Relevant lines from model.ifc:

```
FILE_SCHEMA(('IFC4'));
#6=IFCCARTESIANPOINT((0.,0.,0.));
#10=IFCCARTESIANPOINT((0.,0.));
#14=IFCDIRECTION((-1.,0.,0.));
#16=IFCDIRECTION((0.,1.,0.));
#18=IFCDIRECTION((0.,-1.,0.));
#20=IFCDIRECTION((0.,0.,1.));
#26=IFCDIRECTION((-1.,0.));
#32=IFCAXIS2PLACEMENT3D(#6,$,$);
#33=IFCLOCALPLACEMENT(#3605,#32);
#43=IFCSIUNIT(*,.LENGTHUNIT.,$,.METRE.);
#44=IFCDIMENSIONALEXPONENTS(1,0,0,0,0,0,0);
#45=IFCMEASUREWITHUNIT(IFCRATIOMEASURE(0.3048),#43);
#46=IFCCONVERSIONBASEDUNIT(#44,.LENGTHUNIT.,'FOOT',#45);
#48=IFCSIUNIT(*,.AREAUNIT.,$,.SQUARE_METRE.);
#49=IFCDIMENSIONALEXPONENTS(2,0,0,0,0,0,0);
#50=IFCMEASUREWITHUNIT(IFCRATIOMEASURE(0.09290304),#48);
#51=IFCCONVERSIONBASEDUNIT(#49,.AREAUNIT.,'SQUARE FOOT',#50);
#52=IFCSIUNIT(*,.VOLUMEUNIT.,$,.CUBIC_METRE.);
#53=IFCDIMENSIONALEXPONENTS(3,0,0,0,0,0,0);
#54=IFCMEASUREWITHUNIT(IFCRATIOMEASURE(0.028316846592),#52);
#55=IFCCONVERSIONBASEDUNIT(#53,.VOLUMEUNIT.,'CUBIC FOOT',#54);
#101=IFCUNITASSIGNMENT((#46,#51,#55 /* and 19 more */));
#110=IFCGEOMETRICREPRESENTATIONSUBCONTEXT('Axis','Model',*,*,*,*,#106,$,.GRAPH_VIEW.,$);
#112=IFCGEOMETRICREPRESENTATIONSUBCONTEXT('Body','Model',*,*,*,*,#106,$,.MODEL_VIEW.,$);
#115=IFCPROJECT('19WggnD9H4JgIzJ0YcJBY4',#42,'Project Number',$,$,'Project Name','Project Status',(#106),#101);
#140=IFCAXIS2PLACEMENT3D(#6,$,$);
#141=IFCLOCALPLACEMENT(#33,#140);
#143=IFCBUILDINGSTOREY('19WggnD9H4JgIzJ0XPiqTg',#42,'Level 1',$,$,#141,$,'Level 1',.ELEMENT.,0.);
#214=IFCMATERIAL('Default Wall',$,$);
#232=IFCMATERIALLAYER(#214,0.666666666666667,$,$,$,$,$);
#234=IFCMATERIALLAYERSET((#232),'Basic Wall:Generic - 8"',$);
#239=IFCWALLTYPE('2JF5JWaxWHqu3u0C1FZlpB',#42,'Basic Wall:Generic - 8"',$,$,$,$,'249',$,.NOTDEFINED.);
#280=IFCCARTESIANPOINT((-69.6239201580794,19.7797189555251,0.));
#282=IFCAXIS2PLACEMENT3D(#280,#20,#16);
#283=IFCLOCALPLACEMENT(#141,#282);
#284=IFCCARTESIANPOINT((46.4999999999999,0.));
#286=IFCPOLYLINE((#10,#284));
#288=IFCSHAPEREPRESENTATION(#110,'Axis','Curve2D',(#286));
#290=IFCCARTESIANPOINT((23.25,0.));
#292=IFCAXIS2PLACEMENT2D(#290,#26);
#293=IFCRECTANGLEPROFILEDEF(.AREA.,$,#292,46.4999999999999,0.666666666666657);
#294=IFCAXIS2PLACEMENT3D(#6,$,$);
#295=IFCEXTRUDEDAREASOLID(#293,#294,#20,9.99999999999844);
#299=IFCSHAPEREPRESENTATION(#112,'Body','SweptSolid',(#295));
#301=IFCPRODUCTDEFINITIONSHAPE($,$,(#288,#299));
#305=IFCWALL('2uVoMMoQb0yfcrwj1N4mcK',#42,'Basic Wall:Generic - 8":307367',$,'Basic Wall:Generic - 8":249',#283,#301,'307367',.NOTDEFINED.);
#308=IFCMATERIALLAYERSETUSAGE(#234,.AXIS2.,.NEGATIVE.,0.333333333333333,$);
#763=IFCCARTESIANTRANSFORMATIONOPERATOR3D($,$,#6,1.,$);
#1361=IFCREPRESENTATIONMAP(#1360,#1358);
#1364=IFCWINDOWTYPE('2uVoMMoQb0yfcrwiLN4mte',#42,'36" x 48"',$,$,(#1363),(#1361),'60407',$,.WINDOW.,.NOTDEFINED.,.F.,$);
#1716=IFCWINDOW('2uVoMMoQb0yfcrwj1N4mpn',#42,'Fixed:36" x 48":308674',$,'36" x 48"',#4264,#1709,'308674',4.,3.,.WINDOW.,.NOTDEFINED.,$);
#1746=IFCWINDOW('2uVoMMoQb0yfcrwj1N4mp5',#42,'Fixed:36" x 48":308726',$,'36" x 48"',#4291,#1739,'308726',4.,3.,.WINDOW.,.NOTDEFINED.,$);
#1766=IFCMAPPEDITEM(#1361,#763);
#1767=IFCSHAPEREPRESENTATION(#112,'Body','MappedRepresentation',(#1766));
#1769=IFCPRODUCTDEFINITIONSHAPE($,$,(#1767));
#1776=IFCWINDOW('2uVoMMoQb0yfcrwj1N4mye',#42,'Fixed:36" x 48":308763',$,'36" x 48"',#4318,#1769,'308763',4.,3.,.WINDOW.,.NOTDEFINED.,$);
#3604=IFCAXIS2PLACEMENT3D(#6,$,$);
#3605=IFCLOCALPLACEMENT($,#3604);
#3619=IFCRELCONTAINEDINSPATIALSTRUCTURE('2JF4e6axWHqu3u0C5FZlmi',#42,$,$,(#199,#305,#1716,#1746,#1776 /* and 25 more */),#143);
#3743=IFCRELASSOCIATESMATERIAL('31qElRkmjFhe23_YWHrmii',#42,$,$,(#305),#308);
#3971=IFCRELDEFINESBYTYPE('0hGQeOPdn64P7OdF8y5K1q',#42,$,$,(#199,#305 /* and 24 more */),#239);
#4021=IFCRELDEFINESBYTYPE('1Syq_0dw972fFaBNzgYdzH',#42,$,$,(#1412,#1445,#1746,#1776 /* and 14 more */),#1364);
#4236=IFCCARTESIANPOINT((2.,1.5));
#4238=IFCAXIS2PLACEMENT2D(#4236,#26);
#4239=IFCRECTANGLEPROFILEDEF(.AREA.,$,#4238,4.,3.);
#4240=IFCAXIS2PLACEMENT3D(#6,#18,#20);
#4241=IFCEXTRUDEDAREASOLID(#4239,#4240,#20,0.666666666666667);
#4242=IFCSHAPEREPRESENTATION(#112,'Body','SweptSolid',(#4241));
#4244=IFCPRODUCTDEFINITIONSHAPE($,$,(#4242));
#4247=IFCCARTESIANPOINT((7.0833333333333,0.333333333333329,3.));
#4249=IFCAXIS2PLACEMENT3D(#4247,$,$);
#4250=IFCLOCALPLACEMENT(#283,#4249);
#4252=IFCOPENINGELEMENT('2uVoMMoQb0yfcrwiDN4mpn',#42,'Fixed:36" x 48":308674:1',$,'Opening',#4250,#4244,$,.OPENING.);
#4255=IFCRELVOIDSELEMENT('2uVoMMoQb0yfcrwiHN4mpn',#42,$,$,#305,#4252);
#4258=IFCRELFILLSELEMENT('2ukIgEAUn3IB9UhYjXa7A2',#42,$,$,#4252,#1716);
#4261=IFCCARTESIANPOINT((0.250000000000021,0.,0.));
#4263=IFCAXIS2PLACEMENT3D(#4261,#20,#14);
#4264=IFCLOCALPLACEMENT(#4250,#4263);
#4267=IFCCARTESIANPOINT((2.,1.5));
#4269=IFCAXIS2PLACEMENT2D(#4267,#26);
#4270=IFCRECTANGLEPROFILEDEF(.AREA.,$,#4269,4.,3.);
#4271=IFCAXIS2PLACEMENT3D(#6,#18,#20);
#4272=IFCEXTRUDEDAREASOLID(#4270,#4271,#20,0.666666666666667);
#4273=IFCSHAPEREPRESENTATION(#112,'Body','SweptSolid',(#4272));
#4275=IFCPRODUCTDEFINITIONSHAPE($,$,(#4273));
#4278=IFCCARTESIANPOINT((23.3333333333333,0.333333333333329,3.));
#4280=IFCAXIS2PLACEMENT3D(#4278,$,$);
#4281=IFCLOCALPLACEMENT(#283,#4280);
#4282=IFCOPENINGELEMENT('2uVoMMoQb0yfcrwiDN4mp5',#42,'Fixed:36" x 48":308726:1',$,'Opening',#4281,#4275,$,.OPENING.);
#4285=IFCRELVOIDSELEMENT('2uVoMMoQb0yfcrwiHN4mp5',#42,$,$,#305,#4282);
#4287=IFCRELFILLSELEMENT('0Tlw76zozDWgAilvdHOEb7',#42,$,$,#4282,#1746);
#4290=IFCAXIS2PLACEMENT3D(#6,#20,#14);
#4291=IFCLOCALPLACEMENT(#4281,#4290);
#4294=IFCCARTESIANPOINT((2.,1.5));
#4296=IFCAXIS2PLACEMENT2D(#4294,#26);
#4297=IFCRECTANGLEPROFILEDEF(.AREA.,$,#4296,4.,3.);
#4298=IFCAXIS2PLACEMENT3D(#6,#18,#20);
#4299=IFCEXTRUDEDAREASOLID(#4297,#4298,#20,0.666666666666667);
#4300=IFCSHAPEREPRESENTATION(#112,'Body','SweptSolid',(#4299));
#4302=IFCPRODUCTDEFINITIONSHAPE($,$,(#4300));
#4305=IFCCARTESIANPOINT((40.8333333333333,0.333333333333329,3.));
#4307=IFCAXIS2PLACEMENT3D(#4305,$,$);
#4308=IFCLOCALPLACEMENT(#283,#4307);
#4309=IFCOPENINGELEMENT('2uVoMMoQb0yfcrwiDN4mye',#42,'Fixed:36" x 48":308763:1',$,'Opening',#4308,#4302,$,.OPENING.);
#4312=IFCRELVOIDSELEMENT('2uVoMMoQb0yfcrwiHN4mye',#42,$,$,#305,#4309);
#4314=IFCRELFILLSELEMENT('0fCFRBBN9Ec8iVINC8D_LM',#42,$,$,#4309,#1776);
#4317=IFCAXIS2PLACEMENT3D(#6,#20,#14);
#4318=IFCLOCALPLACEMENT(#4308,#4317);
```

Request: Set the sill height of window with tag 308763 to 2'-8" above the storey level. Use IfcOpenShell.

```python
import numpy as np
import ifcopenshell
import ifcopenshell.api.geometry
import ifcopenshell.geom
import ifcopenshell.util.element
import ifcopenshell.util.placement
import ifcopenshell.util.shape
import ifcopenshell.util.unit

model = ifcopenshell.open("model.ifc")
unit_scale = ifcopenshell.util.unit.calculate_unit_scale(model)

window = model.by_id(1776)
opening = window.FillsVoids[0].RelatingOpeningElement
storey = ifcopenshell.util.element.get_container(window, ifc_class="IfcBuildingStorey")
level = ifcopenshell.util.placement.get_local_placement(storey.ObjectPlacement)[2, 3]

# The opening's origin need not be at the sill, so measure its lowest point.
shape = ifcopenshell.geom.create_shape(ifcopenshell.geom.settings(), opening)
bottom = ifcopenshell.util.shape.get_shape_bottom_elevation(shape, shape.geometry) / unit_scale
dz = level + 32 * 0.0254 / unit_scale - bottom

shift = np.array([0.0, 0.0, dz])
# The window is placed relative to its opening, so it follows when the opening moves.
matrix = ifcopenshell.util.placement.get_local_placement(opening.ObjectPlacement)
matrix[:3, 3] += shift
ifcopenshell.api.geometry.edit_object_placement(
    model, product=opening, matrix=matrix, is_si=False, should_transform_children=True
)

print(f"moved by {dz * unit_scale:+.3f} m")

model.write("model_v2.ifc")
```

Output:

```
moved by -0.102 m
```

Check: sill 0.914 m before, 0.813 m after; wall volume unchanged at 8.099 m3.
